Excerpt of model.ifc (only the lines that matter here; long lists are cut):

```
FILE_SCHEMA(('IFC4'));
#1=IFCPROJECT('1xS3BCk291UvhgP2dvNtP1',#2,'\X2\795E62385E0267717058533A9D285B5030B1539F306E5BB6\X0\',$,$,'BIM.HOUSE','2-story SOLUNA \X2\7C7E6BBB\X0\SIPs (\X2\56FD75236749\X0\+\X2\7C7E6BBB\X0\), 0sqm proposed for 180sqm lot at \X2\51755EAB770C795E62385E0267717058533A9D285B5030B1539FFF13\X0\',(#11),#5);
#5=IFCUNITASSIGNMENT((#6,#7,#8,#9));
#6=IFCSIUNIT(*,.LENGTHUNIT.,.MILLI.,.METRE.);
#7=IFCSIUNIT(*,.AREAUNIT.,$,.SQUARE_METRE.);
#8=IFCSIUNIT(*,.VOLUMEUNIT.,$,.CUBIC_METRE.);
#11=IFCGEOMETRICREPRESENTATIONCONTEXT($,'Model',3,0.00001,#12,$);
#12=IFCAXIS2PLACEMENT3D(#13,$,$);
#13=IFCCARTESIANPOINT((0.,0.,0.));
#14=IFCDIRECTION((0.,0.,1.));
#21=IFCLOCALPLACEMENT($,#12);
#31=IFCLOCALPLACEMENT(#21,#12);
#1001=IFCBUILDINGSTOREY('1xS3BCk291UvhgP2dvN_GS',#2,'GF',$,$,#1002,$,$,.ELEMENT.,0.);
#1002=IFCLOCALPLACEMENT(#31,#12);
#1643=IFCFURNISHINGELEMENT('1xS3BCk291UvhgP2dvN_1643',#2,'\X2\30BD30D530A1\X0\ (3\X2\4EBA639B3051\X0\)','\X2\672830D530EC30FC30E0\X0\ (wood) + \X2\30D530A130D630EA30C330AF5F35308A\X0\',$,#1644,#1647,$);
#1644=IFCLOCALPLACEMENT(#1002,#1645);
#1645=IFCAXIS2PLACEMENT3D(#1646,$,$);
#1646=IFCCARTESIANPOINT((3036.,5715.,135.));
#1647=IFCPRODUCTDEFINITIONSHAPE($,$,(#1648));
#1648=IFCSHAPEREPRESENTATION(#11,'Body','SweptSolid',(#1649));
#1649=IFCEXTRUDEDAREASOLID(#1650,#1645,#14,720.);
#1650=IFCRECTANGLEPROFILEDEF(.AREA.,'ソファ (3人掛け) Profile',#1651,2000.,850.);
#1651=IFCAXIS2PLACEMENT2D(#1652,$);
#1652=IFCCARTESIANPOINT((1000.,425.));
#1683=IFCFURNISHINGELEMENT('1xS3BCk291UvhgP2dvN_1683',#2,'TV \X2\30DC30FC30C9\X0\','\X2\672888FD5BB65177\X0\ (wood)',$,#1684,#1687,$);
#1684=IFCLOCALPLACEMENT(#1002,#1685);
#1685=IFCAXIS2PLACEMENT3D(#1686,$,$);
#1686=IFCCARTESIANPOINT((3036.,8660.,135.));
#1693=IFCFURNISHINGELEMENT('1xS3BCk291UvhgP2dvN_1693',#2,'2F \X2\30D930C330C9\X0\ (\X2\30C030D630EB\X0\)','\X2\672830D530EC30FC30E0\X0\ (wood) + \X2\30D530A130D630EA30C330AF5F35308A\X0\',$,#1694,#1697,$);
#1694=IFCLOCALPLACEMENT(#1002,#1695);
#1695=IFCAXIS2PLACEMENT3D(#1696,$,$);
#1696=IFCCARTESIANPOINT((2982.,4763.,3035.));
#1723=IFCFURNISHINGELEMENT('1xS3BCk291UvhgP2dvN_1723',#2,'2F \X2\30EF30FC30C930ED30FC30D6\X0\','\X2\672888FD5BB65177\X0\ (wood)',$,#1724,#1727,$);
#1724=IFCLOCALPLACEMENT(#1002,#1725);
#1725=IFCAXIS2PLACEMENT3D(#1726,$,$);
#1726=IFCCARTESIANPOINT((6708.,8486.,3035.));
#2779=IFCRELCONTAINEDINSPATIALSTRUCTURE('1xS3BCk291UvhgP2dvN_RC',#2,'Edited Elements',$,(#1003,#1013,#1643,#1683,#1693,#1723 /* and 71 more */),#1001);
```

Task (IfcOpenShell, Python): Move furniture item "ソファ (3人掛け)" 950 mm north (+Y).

```python
import ifcopenshell
import ifcopenshell.api.geometry
import ifcopenshell.util.placement

model = ifcopenshell.open("model.ifc")

item = model.by_guid("1xS3BCk291UvhgP2dvN_1643")
matrix = ifcopenshell.util.placement.get_local_placement(item.ObjectPlacement)
matrix[1, 3] += 950.0
ifcopenshell.api.geometry.edit_object_placement(model, product=item, matrix=matrix, is_si=False)

print(ifcopenshell.util.placement.get_local_placement(item.ObjectPlacement).round(3) + 0.0)

model.write("model_edited.ifc")
```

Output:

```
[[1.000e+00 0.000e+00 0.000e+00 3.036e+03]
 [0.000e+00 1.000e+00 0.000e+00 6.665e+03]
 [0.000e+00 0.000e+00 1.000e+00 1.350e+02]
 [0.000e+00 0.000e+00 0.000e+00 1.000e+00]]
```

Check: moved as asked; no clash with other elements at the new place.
